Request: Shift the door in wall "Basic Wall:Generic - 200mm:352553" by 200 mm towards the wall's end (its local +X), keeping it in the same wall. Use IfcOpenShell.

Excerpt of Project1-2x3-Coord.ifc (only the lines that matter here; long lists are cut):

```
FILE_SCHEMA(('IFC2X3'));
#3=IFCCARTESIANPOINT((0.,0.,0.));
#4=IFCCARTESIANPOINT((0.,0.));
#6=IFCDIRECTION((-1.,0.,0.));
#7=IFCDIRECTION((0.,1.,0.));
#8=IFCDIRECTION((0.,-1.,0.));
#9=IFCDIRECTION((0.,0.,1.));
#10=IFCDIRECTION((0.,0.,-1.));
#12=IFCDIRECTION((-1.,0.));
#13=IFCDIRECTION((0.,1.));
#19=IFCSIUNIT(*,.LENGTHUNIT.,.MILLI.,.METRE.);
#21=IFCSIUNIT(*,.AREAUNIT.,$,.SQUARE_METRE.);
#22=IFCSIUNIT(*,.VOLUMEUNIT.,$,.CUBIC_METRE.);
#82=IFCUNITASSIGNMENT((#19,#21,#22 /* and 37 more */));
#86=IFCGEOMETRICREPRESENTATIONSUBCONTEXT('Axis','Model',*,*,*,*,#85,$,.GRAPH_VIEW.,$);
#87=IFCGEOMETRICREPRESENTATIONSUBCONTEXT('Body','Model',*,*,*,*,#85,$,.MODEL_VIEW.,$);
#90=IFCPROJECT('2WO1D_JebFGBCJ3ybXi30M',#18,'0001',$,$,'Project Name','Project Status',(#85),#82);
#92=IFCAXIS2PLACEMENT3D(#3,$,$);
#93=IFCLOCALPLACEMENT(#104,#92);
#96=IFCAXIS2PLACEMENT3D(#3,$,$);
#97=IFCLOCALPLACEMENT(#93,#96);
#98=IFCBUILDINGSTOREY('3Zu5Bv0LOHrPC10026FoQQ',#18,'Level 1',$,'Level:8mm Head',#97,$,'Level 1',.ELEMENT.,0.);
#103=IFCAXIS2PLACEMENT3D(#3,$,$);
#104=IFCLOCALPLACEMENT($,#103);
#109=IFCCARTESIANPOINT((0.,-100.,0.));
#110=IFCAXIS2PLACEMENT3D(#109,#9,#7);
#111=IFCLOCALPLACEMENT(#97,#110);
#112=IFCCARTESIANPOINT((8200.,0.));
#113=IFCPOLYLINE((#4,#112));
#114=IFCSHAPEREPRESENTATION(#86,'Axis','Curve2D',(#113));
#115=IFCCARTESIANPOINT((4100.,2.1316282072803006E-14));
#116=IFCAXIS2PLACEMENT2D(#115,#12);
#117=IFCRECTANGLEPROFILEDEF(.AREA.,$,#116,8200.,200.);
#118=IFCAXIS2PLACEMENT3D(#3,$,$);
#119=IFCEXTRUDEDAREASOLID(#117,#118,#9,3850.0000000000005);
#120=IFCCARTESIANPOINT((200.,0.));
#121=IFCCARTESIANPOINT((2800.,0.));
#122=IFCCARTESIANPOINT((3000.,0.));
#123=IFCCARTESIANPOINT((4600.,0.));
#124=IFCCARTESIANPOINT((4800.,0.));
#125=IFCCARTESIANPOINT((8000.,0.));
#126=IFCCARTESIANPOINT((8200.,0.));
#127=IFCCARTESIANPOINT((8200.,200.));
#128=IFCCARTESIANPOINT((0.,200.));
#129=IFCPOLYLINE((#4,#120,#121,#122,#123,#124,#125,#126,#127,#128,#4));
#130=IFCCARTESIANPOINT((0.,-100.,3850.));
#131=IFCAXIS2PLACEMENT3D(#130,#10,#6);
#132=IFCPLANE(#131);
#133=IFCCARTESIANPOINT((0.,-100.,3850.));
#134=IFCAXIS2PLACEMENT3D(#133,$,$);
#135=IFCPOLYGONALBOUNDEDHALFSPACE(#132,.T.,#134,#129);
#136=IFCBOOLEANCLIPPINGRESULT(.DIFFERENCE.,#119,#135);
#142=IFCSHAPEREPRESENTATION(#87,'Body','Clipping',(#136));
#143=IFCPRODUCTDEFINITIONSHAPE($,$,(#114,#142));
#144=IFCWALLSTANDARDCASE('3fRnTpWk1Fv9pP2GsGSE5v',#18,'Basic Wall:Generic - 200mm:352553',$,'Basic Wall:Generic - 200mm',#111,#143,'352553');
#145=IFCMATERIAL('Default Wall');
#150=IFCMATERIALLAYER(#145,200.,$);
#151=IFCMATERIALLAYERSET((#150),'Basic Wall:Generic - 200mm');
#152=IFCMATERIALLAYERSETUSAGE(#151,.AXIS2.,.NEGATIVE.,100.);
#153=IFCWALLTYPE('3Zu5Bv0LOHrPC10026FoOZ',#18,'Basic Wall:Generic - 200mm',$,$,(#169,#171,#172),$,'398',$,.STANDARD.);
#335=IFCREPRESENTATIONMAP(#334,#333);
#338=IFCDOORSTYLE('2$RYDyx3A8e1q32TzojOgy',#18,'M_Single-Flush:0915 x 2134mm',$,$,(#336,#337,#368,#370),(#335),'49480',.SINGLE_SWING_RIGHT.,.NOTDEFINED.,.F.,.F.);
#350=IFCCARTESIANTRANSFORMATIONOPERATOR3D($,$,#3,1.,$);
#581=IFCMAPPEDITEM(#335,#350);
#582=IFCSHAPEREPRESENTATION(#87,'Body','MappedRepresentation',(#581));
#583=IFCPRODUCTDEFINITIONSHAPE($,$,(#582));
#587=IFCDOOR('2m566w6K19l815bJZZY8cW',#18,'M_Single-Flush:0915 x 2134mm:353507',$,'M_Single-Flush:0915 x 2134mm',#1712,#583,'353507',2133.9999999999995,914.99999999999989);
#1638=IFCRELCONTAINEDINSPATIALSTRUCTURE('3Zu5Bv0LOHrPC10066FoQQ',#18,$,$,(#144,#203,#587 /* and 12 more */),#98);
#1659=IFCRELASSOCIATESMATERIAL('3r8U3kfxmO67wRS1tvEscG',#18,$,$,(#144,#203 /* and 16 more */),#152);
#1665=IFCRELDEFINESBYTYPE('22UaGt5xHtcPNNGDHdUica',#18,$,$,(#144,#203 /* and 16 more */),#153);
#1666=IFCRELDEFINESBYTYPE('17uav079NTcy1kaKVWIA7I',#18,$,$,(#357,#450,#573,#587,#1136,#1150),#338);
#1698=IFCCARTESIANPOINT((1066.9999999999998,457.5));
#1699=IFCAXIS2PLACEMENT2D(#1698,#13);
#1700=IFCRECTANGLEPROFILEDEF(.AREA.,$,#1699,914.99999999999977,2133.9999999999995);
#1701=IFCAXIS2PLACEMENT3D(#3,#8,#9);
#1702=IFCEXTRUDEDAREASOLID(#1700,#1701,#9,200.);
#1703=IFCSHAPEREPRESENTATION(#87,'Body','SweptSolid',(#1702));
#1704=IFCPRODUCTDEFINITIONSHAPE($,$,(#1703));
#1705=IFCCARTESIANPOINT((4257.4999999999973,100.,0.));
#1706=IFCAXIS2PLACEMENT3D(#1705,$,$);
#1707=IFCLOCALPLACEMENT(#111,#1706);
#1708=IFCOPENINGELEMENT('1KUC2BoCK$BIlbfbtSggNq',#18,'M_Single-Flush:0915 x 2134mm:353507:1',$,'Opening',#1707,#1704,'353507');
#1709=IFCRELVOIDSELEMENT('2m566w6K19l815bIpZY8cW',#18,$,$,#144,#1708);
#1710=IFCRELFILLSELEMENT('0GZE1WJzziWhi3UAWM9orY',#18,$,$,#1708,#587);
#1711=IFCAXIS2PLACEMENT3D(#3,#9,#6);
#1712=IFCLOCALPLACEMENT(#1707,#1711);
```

```python
import ifcopenshell
import ifcopenshell.api.geometry
import ifcopenshell.util.placement
import ifcopenshell.util.unit

model = ifcopenshell.open("Project1-2x3-Coord.ifc")
unit_scale = ifcopenshell.util.unit.calculate_unit_scale(model)

door = model.by_guid("2m566w6K19l815bJZZY8cW")
opening = door.FillsVoids[0].RelatingOpeningElement
wall = opening.VoidsElements[0].RelatingBuildingElement

wall_matrix = ifcopenshell.util.placement.get_local_placement(wall.ObjectPlacement)
shift = wall_matrix[:3, 0] * 0.2 / unit_scale
before = ifcopenshell.util.placement.get_local_placement(door.ObjectPlacement)[:3, 3].copy()

# The door is placed relative to its opening, so it follows when the opening moves.
matrix = ifcopenshell.util.placement.get_local_placement(opening.ObjectPlacement)
matrix[:3, 3] += shift
ifcopenshell.api.geometry.edit_object_placement(
    model, product=opening, matrix=matrix, is_si=False, should_transform_children=True
)

after = ifcopenshell.util.placement.get_local_placement(door.ObjectPlacement)[:3, 3]
print("door moved by", (after - before).round(3) + 0.0)

model.write("Project1-2x3-Coord-out.ifc")
```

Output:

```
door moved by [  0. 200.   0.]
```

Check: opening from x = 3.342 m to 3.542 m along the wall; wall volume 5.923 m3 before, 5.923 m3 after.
